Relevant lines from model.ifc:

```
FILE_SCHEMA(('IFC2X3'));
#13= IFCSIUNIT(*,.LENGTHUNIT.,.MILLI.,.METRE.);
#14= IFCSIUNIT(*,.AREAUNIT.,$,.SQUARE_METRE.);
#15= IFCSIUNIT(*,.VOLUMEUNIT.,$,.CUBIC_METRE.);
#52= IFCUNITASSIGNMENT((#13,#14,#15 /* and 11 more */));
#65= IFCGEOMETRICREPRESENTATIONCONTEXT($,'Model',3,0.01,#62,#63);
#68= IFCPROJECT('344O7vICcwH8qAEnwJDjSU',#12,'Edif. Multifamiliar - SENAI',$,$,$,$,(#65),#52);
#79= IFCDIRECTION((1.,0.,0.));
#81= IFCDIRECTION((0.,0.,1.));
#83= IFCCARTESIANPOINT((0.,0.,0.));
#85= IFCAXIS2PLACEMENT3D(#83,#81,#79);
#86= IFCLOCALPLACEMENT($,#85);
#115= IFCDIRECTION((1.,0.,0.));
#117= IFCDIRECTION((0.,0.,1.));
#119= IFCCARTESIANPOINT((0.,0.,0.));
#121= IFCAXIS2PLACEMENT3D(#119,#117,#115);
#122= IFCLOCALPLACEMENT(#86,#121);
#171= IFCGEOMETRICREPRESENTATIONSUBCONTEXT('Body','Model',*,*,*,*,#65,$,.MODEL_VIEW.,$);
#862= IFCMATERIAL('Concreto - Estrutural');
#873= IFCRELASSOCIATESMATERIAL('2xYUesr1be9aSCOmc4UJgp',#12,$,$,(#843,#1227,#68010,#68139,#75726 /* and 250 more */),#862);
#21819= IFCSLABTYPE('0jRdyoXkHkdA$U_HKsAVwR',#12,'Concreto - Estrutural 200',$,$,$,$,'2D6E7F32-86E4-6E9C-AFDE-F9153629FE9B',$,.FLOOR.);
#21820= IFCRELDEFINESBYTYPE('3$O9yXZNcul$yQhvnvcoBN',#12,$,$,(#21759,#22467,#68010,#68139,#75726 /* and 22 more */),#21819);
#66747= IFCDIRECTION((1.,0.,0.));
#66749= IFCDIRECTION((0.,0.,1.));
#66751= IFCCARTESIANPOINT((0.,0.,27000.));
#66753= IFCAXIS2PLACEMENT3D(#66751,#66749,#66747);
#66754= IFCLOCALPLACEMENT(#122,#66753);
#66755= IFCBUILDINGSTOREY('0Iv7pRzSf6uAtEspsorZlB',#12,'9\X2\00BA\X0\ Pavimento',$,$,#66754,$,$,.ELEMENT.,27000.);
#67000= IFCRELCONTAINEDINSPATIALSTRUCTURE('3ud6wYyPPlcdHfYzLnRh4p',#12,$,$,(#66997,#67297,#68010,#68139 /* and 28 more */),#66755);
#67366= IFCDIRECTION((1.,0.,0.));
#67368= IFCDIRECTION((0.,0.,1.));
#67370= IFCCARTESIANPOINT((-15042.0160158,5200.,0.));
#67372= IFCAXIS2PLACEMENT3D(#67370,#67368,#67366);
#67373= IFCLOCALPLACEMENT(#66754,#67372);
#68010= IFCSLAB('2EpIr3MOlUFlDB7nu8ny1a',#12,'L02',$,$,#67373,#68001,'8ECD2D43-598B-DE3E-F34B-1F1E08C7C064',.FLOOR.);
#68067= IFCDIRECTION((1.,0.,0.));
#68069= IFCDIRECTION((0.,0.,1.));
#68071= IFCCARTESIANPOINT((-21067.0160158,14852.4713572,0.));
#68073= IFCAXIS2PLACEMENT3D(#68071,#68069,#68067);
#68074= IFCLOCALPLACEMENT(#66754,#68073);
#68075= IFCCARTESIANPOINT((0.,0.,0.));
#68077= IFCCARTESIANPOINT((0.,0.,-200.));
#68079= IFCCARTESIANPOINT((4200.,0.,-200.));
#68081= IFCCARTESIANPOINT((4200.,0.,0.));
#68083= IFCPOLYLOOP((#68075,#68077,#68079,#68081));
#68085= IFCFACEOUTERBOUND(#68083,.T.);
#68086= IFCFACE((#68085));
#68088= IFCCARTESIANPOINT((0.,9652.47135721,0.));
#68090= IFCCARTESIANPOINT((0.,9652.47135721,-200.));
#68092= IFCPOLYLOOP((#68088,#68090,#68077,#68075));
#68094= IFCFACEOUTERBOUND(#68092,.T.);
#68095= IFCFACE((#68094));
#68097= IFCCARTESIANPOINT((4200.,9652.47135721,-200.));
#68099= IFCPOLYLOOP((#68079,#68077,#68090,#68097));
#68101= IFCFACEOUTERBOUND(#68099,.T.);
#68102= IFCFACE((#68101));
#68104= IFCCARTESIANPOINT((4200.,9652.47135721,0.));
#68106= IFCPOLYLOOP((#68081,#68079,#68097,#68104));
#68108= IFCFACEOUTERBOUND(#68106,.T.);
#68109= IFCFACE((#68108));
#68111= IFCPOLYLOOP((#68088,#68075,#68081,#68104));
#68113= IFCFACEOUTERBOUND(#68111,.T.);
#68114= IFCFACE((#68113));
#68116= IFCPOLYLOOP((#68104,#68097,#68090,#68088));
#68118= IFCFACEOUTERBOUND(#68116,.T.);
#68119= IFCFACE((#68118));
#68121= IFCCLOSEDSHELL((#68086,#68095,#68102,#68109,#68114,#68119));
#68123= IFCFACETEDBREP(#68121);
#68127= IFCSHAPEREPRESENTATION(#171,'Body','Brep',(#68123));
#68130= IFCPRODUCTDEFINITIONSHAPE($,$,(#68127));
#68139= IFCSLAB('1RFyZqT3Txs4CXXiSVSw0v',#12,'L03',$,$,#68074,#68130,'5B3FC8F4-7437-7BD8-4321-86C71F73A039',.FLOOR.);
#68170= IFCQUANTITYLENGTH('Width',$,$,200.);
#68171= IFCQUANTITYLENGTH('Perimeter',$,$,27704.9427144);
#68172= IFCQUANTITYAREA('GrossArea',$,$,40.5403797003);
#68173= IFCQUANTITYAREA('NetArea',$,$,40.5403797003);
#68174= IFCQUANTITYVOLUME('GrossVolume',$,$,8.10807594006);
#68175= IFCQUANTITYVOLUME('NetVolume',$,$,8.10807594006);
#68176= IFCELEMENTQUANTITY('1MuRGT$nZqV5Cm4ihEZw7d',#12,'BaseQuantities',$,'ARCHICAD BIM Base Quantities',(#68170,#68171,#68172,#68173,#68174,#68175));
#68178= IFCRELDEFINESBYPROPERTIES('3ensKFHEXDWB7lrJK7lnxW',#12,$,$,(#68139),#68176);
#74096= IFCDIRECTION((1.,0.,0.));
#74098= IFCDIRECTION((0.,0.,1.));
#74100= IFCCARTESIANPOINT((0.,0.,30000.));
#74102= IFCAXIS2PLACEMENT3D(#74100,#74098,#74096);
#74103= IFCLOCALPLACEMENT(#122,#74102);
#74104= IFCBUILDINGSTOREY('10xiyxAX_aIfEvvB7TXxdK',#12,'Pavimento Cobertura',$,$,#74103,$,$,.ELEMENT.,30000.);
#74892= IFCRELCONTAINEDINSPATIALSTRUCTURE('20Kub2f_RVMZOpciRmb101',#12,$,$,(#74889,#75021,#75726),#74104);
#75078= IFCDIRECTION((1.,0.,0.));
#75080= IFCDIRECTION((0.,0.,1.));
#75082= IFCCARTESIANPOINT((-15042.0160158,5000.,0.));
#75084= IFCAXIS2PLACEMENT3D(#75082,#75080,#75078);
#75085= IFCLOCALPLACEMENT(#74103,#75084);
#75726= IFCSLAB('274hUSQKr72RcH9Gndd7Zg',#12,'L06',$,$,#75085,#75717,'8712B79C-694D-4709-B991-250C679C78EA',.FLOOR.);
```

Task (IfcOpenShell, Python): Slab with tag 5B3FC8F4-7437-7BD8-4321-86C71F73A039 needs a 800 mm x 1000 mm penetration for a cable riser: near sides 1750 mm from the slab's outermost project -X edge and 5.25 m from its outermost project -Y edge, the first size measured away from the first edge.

```python
import numpy as np
import ifcopenshell
import ifcopenshell.api.feature
import ifcopenshell.api.geometry
import ifcopenshell.api.pset
import ifcopenshell.api.root
import ifcopenshell.geom
import ifcopenshell.util.element
import ifcopenshell.util.placement
import ifcopenshell.util.representation
import ifcopenshell.util.shape
import ifcopenshell.util.unit

model = ifcopenshell.open("model.ifc")
unit_scale = ifcopenshell.util.unit.calculate_unit_scale(model)
area_scale = ifcopenshell.util.unit.calculate_unit_scale(model, "AREAUNIT")
volume_scale = ifcopenshell.util.unit.calculate_unit_scale(model, "VOLUMEUNIT")
settings = ifcopenshell.geom.settings()


def volume(element):
    """Net volume in cubic metres, openings subtracted."""
    shape = ifcopenshell.geom.create_shape(settings, element)
    return ifcopenshell.util.shape.get_volume(shape.geometry)


slab = model.by_guid("1RFyZqT3Txs4CXXiSVSw0v")
before = volume(slab)

# Extent in the slab's own axes, in metres. The edges named are its -X and -Y sides.
slab_shape = ifcopenshell.geom.create_shape(settings, slab)
vertices = ifcopenshell.util.shape.get_vertices(slab_shape.geometry)
x_min, y_min, bottom = vertices.min(axis=0)
top = vertices[:, 2].max()

opening = ifcopenshell.api.root.create_entity(model, ifc_class="IfcOpeningElement", name="Cable riser opening")
context = ifcopenshell.util.representation.get_context(model, "Model", "Body", "MODEL_VIEW")
width, depth = 0.8, 1
outline = [(0.0, 0.0), (width, 0.0), (width, depth), (0.0, depth), (0.0, 0.0)]
# Overshoot both faces by 50 mm so the cut is clean.
shape = ifcopenshell.api.geometry.add_slab_representation(
    model, context=context, depth=top - bottom + 0.1, polyline=outline
)
ifcopenshell.api.geometry.assign_representation(model, product=opening, representation=shape)

matrix = ifcopenshell.util.placement.get_local_placement(slab.ObjectPlacement)
matrix[:, 3] = matrix @ np.append(np.array([x_min + 1.75, y_min + 5.25, bottom - 0.05]) / unit_scale, 1.0)
ifcopenshell.api.geometry.edit_object_placement(model, product=opening, matrix=matrix, is_si=False)
ifcopenshell.api.feature.add_feature(model, feature=opening, element=slab)

after = volume(slab)

# Update the slab's stored quantities.
qto = model.by_id(ifcopenshell.util.element.get_pset(slab, "BaseQuantities", should_inherit=False)["id"])
ifcopenshell.api.pset.edit_qto(model, qto=qto, properties={
    "NetArea": after / (top - bottom) / area_scale,
    "NetVolume": after / volume_scale,
})

print(f"slab volume {before:.3f} -> {after:.3f} m3")

model.write("model_rev.ifc")
```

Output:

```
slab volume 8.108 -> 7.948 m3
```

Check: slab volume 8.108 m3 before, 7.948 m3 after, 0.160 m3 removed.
